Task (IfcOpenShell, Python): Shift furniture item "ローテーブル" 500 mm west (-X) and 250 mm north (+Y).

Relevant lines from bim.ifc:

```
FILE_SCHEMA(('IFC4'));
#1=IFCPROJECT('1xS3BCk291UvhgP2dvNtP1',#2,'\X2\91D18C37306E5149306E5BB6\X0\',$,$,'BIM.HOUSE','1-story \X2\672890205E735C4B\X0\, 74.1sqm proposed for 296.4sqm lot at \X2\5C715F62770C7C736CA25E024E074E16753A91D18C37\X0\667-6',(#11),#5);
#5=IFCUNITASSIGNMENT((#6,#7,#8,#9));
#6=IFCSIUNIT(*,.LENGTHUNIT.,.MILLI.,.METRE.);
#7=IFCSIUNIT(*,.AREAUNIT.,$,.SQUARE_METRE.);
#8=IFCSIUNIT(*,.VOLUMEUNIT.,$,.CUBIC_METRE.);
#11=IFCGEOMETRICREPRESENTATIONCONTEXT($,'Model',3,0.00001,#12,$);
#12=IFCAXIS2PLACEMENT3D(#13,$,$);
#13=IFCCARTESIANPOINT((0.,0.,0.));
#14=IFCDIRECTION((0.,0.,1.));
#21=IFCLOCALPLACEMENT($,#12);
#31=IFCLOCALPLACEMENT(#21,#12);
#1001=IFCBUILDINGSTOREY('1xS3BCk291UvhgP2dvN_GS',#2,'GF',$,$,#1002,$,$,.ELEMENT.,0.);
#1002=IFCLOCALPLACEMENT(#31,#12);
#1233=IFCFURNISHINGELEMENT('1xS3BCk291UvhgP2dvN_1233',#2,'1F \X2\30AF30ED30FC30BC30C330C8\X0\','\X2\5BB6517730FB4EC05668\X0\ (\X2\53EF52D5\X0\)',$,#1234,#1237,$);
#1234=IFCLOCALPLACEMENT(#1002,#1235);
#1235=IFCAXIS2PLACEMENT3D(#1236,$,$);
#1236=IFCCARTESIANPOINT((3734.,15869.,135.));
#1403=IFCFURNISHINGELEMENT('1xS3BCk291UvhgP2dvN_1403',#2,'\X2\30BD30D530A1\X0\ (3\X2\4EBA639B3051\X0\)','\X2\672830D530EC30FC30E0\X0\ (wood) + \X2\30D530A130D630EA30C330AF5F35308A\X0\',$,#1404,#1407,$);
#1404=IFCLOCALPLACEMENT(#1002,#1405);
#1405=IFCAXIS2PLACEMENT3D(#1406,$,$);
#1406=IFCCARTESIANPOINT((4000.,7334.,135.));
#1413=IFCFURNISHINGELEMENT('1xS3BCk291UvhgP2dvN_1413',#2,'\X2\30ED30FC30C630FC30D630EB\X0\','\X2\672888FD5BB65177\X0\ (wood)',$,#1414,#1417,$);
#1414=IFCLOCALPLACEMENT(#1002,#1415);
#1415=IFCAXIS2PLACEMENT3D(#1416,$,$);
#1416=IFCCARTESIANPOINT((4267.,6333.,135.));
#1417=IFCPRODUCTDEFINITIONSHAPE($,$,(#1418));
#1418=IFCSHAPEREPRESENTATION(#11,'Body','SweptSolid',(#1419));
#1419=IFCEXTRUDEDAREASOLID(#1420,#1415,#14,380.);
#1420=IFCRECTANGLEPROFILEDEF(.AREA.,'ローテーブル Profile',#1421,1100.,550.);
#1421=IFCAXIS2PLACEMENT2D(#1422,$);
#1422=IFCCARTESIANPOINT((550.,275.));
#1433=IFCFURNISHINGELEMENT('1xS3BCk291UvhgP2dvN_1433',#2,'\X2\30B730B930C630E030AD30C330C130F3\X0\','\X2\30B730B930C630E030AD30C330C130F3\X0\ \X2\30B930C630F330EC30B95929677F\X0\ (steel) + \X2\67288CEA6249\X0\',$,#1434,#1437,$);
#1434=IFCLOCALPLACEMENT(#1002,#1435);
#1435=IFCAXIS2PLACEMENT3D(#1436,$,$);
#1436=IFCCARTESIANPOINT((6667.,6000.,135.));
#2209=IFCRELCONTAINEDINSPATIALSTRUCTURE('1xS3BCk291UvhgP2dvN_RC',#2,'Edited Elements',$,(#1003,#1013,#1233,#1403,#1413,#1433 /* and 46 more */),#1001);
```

```python
import ifcopenshell
import ifcopenshell.api.geometry
import ifcopenshell.util.placement

model = ifcopenshell.open("bim.ifc")

item = model.by_guid("1xS3BCk291UvhgP2dvN_1413")
matrix = ifcopenshell.util.placement.get_local_placement(item.ObjectPlacement)
matrix[0, 3] -= 500.0
matrix[1, 3] += 250.0
ifcopenshell.api.geometry.edit_object_placement(model, product=item, matrix=matrix, is_si=False)

print(ifcopenshell.util.placement.get_local_placement(item.ObjectPlacement).round(3) + 0.0)

model.write("bim_updated.ifc")
```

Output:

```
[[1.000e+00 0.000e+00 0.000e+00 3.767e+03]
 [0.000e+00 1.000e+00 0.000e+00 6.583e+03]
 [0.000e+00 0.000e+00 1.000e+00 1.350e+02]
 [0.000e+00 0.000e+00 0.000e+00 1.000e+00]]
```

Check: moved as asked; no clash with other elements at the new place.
